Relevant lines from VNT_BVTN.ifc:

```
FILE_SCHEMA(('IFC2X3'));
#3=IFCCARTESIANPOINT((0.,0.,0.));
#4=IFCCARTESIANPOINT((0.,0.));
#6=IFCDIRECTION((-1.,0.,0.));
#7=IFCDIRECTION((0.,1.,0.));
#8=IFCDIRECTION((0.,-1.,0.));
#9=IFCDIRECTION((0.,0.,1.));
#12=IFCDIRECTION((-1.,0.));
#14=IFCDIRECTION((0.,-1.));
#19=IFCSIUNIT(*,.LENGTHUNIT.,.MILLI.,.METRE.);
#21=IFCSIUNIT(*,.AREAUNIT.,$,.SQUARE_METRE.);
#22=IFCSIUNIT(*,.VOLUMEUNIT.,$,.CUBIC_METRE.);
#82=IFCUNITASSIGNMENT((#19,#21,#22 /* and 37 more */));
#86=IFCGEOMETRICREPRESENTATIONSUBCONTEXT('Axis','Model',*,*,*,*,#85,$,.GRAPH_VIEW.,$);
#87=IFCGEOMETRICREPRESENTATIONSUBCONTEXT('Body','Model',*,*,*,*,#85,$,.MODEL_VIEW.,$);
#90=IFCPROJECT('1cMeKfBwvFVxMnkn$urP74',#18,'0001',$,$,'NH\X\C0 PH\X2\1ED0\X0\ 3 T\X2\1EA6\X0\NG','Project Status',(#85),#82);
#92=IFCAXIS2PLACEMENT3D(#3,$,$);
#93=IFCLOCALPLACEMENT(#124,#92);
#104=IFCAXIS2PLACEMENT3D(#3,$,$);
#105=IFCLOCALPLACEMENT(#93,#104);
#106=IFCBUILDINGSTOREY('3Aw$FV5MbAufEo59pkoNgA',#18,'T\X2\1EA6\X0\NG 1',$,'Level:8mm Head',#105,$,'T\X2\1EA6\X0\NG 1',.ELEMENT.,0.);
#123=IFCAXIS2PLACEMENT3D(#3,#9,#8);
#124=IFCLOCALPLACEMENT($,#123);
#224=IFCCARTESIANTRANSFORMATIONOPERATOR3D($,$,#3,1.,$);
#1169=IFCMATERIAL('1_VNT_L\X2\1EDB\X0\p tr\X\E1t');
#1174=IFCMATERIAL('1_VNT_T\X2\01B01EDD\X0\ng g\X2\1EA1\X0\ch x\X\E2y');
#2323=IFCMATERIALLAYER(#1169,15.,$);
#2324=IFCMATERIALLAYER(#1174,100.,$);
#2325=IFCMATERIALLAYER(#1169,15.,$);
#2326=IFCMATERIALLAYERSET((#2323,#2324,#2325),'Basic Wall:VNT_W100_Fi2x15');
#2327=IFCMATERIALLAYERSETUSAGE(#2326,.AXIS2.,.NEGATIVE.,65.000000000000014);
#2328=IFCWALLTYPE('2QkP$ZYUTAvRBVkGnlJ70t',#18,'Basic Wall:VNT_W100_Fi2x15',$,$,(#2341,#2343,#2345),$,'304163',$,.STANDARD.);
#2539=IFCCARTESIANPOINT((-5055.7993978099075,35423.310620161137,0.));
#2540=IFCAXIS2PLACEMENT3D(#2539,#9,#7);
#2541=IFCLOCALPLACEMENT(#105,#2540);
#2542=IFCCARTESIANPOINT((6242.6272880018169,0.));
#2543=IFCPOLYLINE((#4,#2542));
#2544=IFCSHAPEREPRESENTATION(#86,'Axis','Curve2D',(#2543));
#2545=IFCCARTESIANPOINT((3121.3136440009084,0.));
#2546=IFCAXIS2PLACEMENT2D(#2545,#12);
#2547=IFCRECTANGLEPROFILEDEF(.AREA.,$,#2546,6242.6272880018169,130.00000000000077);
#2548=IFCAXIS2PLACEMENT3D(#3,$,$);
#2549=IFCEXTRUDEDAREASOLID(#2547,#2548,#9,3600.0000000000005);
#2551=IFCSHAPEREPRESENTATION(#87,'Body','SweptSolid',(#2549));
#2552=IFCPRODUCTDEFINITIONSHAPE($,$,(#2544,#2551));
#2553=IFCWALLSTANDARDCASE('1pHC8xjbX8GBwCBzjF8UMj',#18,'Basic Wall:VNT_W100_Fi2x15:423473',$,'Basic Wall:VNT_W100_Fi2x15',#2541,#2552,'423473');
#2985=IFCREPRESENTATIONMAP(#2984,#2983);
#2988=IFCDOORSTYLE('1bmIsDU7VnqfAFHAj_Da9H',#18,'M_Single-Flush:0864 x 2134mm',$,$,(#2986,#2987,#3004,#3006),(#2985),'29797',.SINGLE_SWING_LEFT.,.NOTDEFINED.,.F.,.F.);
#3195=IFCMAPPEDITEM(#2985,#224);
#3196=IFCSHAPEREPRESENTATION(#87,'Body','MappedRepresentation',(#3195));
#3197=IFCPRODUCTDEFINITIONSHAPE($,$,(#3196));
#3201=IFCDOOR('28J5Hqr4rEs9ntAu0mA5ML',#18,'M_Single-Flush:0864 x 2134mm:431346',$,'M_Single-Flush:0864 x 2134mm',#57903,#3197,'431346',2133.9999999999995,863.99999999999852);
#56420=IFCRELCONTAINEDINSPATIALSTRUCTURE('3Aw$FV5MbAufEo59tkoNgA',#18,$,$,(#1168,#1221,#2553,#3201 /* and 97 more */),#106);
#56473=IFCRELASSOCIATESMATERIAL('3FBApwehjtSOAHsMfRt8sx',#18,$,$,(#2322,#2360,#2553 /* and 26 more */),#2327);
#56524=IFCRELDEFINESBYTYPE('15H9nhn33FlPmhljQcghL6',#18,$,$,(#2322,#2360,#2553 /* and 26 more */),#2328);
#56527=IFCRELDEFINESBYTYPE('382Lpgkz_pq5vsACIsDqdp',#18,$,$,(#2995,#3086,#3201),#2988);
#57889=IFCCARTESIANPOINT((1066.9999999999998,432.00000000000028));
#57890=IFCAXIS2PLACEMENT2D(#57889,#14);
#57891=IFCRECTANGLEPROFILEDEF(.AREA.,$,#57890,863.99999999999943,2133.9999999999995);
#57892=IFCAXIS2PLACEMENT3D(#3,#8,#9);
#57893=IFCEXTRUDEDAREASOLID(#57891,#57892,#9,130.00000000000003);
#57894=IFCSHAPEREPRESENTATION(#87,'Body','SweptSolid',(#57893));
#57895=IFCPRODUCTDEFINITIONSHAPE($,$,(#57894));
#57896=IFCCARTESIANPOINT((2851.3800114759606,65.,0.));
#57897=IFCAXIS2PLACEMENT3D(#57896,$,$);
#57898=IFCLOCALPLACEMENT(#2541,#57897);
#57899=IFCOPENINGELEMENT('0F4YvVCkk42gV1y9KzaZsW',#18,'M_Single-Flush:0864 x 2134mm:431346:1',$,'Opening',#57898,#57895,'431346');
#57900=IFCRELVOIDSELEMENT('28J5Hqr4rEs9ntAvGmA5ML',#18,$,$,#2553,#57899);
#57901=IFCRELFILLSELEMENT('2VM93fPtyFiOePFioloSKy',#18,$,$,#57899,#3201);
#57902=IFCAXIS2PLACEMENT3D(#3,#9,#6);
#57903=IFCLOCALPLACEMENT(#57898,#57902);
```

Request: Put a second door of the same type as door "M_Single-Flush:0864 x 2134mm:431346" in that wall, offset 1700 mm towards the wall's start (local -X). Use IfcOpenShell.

```python
import ifcopenshell
import ifcopenshell.api.feature
import ifcopenshell.api.geometry
import ifcopenshell.api.root
import ifcopenshell.geom
import ifcopenshell.util.element
import ifcopenshell.util.placement
import ifcopenshell.util.shape
import ifcopenshell.util.unit

model = ifcopenshell.open("VNT_BVTN.ifc")
unit_scale = ifcopenshell.util.unit.calculate_unit_scale(model)
settings = ifcopenshell.geom.settings()


def volume(element):
    """Net volume in cubic metres, openings subtracted."""
    shape = ifcopenshell.geom.create_shape(settings, element)
    return ifcopenshell.util.shape.get_volume(shape.geometry)


def reuse_history(source, copy):
    """copy_class also copies each property set's owner history, people and application; keep the originals."""
    for rel in copy.IsDefinedBy:
        if rel.is_a("IfcRelDefinesByProperties") and (history := rel.RelatingPropertyDefinition.OwnerHistory):
            rel.RelatingPropertyDefinition.OwnerHistory = source.OwnerHistory
            ifcopenshell.util.element.remove_deep2(model, history)


door = model.by_guid("28J5Hqr4rEs9ntAu0mA5ML")
opening = door.FillsVoids[0].RelatingOpeningElement
wall = opening.VoidsElements[0].RelatingBuildingElement
before = volume(wall)
shift = ifcopenshell.util.placement.get_local_placement(wall.ObjectPlacement)[:3, 0] * -1.7 / unit_scale

# copy_class copies the void relationship, type, container and properties, but no geometry.
new_opening = ifcopenshell.api.root.copy_class(model, product=opening)
new_opening.Representation = ifcopenshell.util.element.copy_deep(
    model, opening.Representation, exclude=["IfcGeometricRepresentationContext", "IfcRepresentationMap"]
)
new_opening.Name = "M_Single-Flush:0864 x 2134mm"
new_opening.Tag = None
new_door = ifcopenshell.api.root.copy_class(model, product=door)
new_door.Representation = ifcopenshell.util.element.copy_deep(
    model, door.Representation, exclude=["IfcGeometricRepresentationContext", "IfcRepresentationMap"]
)
new_door.Name = "M_Single-Flush:0864 x 2134mm"
new_door.Tag = None
reuse_history(door, new_door)
fills = ifcopenshell.api.feature.add_filling(model, opening=new_opening, element=new_door)
fills.OwnerHistory = new_door.OwnerHistory  # required in IFC2X3

for old, new in ((opening, new_opening), (door, new_door)):
    matrix = ifcopenshell.util.placement.get_local_placement(old.ObjectPlacement)
    matrix[:3, 3] += shift
    ifcopenshell.api.geometry.edit_object_placement(model, product=new, matrix=matrix, is_si=False)

after = volume(wall)

print(f"wall volume {before:.3f} -> {after:.3f} m3")

model.write("VNT_BVTN-out.ifc")
```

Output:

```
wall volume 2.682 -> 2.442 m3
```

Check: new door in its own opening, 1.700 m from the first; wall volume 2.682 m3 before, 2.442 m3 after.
